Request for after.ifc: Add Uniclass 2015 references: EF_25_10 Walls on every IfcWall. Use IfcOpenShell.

First a look at what the model holds.

```python
import ifcopenshell

model = ifcopenshell.open("after.ifc")
print(model.schema)
print("classifications:", [c.Name for c in model.by_type("IfcClassification")])
for ifc_class in ("IfcDoor", "IfcRoof", "IfcStair", "IfcWall", "IfcWindow"):
    print(ifc_class, len(model.by_type(ifc_class)))
```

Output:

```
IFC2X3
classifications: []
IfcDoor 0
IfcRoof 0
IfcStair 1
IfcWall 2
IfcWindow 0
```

```python
import ifcopenshell
import ifcopenshell.api.classification

model = ifcopenshell.open("after.ifc")

# IFC2X3 requires Source and Edition and has no link from the project to the system.
system = model.create_entity("IfcClassification", Source="NBS", Edition="2015", Name="Uniclass 2015")

codes = {
    "IfcWall": ("EF_25_10", "Walls"),
}
for ifc_class, (code, name) in codes.items():
    products = model.by_type(ifc_class)
    ifcopenshell.api.classification.add_reference(
        model, products=products, classification=system, identification=code, name=name
    )
    print(code, len(products))

model.write("after_edited.ifc")
```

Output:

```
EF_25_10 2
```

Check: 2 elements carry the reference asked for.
